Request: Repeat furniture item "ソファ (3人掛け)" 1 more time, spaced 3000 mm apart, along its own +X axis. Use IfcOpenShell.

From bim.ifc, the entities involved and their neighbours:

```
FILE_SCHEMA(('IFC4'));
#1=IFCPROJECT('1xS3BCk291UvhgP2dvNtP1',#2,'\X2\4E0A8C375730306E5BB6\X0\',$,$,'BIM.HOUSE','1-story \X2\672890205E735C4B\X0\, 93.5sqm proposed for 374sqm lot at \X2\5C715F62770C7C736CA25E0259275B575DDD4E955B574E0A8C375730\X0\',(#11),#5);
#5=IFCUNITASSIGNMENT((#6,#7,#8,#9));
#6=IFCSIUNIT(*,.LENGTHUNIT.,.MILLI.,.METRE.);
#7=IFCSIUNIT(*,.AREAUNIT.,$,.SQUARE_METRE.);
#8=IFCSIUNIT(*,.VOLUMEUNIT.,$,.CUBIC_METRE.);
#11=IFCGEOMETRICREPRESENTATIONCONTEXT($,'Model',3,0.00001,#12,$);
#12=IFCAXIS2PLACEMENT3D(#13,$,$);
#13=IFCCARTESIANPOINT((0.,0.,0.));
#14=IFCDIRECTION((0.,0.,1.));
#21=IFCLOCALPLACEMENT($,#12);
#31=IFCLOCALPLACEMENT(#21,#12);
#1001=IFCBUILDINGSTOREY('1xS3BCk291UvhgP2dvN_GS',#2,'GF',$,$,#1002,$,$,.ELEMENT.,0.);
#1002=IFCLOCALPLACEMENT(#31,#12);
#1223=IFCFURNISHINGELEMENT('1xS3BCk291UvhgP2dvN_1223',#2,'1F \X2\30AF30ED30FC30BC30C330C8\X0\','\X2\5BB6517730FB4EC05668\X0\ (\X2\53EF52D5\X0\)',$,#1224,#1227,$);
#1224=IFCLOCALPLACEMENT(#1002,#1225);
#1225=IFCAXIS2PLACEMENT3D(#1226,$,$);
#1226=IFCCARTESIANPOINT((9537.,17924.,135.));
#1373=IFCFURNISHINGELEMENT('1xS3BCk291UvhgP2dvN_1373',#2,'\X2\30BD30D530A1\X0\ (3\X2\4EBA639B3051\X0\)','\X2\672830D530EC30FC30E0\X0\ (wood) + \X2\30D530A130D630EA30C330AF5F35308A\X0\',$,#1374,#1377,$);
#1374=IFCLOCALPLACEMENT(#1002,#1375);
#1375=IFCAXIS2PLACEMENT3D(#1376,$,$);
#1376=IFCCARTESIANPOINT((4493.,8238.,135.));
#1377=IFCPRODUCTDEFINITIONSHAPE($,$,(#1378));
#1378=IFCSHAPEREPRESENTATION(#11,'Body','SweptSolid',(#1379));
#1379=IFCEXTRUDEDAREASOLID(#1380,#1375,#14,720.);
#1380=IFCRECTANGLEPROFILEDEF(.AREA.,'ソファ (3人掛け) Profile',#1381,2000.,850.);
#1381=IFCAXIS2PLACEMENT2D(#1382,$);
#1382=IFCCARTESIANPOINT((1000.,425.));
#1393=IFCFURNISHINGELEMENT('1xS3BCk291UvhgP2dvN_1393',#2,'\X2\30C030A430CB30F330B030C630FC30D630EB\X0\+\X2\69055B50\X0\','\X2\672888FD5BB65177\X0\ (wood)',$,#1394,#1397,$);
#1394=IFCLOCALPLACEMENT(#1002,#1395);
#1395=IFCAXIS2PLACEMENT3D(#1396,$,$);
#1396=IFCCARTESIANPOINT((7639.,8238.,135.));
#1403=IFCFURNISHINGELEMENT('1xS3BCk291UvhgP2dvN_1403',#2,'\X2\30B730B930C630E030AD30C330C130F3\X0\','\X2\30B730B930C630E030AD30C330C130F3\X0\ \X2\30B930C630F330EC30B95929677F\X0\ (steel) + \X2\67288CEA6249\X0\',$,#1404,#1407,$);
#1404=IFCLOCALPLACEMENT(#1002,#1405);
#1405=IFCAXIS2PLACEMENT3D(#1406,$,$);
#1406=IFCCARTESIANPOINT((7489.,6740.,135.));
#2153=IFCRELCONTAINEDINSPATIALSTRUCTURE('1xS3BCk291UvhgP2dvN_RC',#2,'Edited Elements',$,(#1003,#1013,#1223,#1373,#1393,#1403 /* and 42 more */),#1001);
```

```python
import ifcopenshell
import ifcopenshell.api.geometry
import ifcopenshell.api.root
import ifcopenshell.util.element
import ifcopenshell.util.placement
import ifcopenshell.util.unit

model = ifcopenshell.open("bim.ifc")
unit_scale = ifcopenshell.util.unit.calculate_unit_scale(model)


def reuse_history(source, copy):
    """copy_class also copies each property set's owner history, people and application; keep the originals."""
    for rel in copy.IsDefinedBy:
        if rel.is_a("IfcRelDefinesByProperties") and (history := rel.RelatingPropertyDefinition.OwnerHistory):
            rel.RelatingPropertyDefinition.OwnerHistory = source.OwnerHistory
            ifcopenshell.util.element.remove_deep2(model, history)


source = model.by_id(1373)
base = ifcopenshell.util.placement.get_local_placement(source.ObjectPlacement)
step = base[:3, 0] * 3 / unit_scale

for i in range(1, 2):
    copy = ifcopenshell.api.root.copy_class(model, product=source)
    copy.Representation = ifcopenshell.util.element.copy_deep(
        model, source.Representation, exclude=["IfcGeometricRepresentationContext", "IfcRepresentationMap"]
    )
    reuse_history(source, copy)
    matrix = base.copy()
    matrix[:3, 3] += i * step
    print("added at", matrix[:3, 3].round(3) + 0.0)
    ifcopenshell.api.geometry.edit_object_placement(model, product=copy, matrix=matrix, is_si=False)

model.write("bim_v2.ifc")
```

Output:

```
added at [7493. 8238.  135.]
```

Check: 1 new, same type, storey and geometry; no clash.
